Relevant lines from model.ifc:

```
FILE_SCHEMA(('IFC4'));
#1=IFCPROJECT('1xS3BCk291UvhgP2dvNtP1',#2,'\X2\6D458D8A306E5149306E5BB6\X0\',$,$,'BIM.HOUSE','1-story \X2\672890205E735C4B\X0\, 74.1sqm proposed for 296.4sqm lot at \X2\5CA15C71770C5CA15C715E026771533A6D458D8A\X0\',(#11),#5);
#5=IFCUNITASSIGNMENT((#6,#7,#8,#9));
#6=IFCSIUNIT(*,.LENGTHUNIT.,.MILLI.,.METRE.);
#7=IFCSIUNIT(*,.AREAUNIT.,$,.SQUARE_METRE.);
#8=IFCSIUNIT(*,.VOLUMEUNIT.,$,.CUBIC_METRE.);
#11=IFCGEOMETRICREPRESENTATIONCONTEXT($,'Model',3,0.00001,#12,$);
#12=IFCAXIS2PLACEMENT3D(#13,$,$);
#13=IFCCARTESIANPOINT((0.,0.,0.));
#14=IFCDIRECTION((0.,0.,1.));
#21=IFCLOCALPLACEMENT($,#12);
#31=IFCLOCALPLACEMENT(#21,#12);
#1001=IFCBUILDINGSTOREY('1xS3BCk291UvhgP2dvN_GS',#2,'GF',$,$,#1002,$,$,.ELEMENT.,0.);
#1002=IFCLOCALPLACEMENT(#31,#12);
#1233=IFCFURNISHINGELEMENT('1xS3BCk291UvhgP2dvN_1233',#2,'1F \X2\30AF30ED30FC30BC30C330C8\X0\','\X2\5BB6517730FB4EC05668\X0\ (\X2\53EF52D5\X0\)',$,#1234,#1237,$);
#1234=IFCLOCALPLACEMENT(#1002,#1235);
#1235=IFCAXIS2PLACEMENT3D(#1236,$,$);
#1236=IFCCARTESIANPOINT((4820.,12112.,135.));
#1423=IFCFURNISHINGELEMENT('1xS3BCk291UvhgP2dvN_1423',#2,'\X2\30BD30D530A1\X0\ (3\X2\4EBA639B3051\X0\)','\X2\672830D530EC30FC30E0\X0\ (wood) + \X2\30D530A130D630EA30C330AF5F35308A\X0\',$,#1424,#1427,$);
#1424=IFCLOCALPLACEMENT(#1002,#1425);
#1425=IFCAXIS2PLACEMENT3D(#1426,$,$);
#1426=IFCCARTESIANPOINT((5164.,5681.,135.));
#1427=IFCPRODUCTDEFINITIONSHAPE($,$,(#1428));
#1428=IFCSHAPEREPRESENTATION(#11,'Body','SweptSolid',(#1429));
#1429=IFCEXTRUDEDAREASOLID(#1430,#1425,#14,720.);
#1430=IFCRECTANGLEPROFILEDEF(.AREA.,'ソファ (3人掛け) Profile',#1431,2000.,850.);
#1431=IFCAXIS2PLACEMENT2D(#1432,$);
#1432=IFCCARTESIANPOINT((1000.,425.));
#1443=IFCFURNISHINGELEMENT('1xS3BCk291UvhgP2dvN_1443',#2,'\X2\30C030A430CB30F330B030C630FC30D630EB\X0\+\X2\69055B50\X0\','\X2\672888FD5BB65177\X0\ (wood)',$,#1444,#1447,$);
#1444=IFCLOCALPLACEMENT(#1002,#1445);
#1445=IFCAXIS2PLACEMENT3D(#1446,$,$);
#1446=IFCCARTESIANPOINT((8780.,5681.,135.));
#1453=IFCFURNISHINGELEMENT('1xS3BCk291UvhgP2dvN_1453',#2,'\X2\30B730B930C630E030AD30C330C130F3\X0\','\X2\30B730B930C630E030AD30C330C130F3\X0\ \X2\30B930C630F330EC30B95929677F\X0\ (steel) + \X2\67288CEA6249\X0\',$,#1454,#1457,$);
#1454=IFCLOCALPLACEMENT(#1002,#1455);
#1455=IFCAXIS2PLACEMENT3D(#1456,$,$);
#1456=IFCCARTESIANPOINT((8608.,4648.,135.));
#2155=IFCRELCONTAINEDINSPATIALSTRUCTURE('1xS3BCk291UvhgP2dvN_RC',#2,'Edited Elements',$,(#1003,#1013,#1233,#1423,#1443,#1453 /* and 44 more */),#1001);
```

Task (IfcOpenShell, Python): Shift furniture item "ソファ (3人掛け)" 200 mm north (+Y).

```python
import ifcopenshell
import ifcopenshell.api.geometry
import ifcopenshell.util.placement
import ifcopenshell.util.unit

model = ifcopenshell.open("model.ifc")
unit_scale = ifcopenshell.util.unit.calculate_unit_scale(model)

item = model.by_guid("1xS3BCk291UvhgP2dvN_1423")
matrix = ifcopenshell.util.placement.get_local_placement(item.ObjectPlacement)
matrix[1, 3] += 0.2 / unit_scale
ifcopenshell.api.geometry.edit_object_placement(model, product=item, matrix=matrix, is_si=False)

print(ifcopenshell.util.placement.get_local_placement(item.ObjectPlacement).round(3) + 0.0)

model.write("model_v2.ifc")
```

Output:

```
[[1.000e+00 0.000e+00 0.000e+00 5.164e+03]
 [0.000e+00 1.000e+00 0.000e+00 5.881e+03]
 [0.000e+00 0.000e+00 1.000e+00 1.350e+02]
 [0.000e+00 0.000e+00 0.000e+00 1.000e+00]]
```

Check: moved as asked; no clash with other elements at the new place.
